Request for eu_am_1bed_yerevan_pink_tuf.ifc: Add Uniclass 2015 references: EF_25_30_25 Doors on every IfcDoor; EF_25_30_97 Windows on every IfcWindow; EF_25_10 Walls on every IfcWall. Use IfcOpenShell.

First a look at what the model holds.

```python
import ifcopenshell

model = ifcopenshell.open("eu_am_1bed_yerevan_pink_tuf.ifc")
print(model.schema)
print("classifications:", [c.Name for c in model.by_type("IfcClassification")])
for ifc_class in ("IfcDoor", "IfcRoof", "IfcStair", "IfcWall", "IfcWindow"):
    print(ifc_class, len(model.by_type(ifc_class)))
```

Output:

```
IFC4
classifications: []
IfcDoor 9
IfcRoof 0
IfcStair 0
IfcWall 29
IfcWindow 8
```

```python
import ifcopenshell
import ifcopenshell.api.classification

model = ifcopenshell.open("eu_am_1bed_yerevan_pink_tuf.ifc")

system = ifcopenshell.api.classification.add_classification(model, classification="Uniclass 2015")

codes = {
    "IfcDoor": ("EF_25_30_25", "Doors"),
    "IfcWindow": ("EF_25_30_97", "Windows"),
    "IfcWall": ("EF_25_10", "Walls"),
}
for ifc_class, (code, name) in codes.items():
    products = model.by_type(ifc_class)
    ifcopenshell.api.classification.add_reference(
        model, products=products, classification=system, identification=code, name=name
    )
    print(code, len(products))

model.write("eu_am_1bed_yerevan_pink_tuf_v2.ifc")
```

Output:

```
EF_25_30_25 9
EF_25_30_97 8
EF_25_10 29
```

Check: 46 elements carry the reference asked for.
